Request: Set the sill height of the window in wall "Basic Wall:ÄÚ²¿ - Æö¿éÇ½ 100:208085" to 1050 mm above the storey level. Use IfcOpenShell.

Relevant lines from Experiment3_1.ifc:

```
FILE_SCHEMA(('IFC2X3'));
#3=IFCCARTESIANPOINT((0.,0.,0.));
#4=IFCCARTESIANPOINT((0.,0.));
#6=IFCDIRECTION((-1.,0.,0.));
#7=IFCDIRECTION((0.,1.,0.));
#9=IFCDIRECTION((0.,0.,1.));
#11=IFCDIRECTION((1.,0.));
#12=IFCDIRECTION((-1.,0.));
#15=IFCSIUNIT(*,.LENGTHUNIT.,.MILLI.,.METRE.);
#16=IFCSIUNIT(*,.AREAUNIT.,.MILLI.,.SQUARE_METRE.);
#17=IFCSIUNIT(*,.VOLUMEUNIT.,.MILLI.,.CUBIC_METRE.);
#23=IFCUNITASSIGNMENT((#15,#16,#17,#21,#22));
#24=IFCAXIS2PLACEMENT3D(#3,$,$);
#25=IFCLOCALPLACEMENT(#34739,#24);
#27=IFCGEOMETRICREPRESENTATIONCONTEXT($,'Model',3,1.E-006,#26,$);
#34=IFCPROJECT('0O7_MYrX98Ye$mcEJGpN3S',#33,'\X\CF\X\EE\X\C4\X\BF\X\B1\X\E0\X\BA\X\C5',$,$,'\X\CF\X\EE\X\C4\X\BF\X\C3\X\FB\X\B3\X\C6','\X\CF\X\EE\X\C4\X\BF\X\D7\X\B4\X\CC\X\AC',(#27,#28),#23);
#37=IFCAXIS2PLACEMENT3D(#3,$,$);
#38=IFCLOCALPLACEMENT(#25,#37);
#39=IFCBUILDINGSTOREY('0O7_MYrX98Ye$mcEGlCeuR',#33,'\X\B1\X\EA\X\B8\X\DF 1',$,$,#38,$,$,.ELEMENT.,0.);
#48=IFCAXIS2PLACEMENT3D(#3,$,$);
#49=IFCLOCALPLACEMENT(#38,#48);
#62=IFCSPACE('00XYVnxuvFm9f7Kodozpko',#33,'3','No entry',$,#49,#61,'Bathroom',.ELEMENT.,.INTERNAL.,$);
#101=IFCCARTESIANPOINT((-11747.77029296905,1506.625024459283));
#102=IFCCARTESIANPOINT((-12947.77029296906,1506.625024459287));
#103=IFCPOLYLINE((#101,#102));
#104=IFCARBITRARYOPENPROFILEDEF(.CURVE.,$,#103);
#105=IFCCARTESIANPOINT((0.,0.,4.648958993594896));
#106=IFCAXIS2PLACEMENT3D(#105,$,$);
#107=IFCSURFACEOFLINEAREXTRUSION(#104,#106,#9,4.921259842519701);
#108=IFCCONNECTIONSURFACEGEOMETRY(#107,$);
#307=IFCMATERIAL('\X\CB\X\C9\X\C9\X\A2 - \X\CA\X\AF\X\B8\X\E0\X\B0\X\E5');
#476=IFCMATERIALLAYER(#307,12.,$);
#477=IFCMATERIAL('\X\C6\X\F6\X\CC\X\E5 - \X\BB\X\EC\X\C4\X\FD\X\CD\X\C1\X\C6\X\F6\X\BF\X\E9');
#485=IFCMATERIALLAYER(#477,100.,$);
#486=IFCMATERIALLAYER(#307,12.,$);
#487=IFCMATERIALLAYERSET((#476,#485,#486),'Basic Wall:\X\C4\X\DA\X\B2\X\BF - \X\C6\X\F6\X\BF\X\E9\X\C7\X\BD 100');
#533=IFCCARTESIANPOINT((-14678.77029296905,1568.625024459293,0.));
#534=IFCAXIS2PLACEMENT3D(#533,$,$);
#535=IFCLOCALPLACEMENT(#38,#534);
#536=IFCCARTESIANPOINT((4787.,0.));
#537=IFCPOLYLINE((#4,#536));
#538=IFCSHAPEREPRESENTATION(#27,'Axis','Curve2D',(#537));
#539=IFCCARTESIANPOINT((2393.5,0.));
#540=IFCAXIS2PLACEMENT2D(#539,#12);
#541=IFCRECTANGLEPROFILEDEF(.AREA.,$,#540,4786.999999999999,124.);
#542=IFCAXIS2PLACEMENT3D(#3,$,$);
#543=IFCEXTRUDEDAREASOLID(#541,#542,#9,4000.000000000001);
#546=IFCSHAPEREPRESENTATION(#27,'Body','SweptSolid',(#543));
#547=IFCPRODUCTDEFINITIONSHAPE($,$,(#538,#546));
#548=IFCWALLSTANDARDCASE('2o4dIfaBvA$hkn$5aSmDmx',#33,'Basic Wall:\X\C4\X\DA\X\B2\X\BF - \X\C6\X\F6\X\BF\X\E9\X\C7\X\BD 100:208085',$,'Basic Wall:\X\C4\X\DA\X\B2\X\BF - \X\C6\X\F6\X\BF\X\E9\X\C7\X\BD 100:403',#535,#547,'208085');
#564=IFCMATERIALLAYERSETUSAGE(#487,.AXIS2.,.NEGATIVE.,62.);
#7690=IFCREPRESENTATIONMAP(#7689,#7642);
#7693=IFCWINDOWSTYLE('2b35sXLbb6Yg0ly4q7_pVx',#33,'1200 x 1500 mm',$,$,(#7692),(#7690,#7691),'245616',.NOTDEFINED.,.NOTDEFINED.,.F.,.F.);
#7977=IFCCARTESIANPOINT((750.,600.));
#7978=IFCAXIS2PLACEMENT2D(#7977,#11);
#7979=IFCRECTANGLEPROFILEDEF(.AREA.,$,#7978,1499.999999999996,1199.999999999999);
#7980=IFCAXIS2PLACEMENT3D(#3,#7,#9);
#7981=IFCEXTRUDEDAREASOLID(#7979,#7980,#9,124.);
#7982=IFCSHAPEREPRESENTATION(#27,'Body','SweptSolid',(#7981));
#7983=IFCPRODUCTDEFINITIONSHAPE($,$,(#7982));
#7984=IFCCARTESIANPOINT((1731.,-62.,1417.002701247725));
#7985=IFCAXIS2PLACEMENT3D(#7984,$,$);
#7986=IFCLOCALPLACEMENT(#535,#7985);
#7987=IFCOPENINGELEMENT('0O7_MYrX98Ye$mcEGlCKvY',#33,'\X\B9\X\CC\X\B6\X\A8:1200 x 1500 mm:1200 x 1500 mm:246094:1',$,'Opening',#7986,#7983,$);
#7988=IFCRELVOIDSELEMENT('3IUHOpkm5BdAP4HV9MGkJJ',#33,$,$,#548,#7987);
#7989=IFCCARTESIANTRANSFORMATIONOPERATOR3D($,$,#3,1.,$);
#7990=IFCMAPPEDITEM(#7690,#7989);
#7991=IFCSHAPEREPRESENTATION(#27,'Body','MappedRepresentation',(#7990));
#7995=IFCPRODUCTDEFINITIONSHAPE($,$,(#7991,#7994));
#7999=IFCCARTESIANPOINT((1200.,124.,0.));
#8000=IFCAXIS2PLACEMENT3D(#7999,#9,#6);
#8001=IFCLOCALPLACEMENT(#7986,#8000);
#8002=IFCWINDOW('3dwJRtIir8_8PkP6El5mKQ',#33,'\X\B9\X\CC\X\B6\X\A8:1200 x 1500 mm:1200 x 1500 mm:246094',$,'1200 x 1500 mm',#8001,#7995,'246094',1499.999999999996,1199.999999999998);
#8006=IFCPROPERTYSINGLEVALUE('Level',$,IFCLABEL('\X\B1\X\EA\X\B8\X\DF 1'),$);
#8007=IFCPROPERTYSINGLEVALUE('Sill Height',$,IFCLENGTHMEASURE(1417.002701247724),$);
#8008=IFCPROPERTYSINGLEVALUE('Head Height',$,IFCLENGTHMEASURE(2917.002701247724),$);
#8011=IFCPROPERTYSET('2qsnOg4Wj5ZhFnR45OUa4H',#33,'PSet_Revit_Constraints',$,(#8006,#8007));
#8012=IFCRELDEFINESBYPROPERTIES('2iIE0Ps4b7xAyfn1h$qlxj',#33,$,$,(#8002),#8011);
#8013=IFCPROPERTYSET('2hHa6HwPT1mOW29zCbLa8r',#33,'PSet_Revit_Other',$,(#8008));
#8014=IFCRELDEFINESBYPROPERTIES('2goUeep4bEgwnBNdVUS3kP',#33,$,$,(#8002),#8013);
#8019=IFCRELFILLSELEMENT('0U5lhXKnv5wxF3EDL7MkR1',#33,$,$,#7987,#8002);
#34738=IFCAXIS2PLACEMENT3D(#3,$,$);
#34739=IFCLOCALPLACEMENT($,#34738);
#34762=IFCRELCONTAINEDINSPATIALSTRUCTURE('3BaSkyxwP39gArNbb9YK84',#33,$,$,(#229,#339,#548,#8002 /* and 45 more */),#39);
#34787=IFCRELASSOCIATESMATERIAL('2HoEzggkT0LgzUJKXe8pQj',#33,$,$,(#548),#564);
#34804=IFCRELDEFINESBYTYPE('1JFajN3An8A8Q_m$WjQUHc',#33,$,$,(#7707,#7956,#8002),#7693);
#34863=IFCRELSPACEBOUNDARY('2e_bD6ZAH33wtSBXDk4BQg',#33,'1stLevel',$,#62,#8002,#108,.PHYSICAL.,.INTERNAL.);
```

```python
import numpy as np
import ifcopenshell
import ifcopenshell.api.geometry
import ifcopenshell.api.pset
import ifcopenshell.geom
import ifcopenshell.util.element
import ifcopenshell.util.placement
import ifcopenshell.util.shape
import ifcopenshell.util.unit

model = ifcopenshell.open("Experiment3_1.ifc")
unit_scale = ifcopenshell.util.unit.calculate_unit_scale(model)

window = model.by_guid("3dwJRtIir8_8PkP6El5mKQ")
opening = window.FillsVoids[0].RelatingOpeningElement
storey = ifcopenshell.util.element.get_container(window, ifc_class="IfcBuildingStorey")
level = ifcopenshell.util.placement.get_local_placement(storey.ObjectPlacement)[2, 3]

# The opening's origin need not be at the sill, so measure its lowest point.
shape = ifcopenshell.geom.create_shape(ifcopenshell.geom.settings(), opening)
bottom = ifcopenshell.util.shape.get_shape_bottom_elevation(shape, shape.geometry) / unit_scale
dz = level + 1.05 / unit_scale - bottom

shift = np.array([0.0, 0.0, dz])
# The window is placed relative to its opening, so it follows when the opening moves.
matrix = ifcopenshell.util.placement.get_local_placement(opening.ObjectPlacement)
matrix[:3, 3] += shift
ifcopenshell.api.geometry.edit_object_placement(
    model, product=opening, matrix=matrix, is_si=False, should_transform_children=True
)

# Space boundary surfaces are stored in each space's coordinates; move them too.
for rel in window.ProvidesBoundaries:
    if not rel.ConnectionGeometry:
        continue
    surface = rel.ConnectionGeometry.SurfaceOnRelatingElement
    space_matrix = ifcopenshell.util.placement.get_local_placement(rel.RelatingSpace.ObjectPlacement)
    point = np.array(surface.Position.Location.Coordinates) + space_matrix[:3, :3].T @ shift
    surface.Position = model.createIfcAxis2Placement3D(
        model.createIfcCartesianPoint(point.tolist()), surface.Position.Axis, surface.Position.RefDirection
    )

# Keep the stored heights in step.
pset = model.by_id(ifcopenshell.util.element.get_pset(window, "PSet_Revit_Constraints", should_inherit=False)["id"])
ifcopenshell.api.pset.edit_pset(model, pset=pset, properties={
    "Sill Height": model.create_entity("IfcLengthMeasure", ifcopenshell.util.element.get_pset(window, "PSet_Revit_Constraints", "Sill Height") + dz),
})
pset = model.by_id(ifcopenshell.util.element.get_pset(window, "PSet_Revit_Other", should_inherit=False)["id"])
ifcopenshell.api.pset.edit_pset(model, pset=pset, properties={
    "Head Height": model.create_entity("IfcLengthMeasure", ifcopenshell.util.element.get_pset(window, "PSet_Revit_Other", "Head Height") + dz),
})

print(f"moved by {dz * unit_scale:+.3f} m")

model.write("Experiment3_1_v2.ifc")
```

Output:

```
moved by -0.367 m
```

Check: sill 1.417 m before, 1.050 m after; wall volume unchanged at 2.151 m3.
